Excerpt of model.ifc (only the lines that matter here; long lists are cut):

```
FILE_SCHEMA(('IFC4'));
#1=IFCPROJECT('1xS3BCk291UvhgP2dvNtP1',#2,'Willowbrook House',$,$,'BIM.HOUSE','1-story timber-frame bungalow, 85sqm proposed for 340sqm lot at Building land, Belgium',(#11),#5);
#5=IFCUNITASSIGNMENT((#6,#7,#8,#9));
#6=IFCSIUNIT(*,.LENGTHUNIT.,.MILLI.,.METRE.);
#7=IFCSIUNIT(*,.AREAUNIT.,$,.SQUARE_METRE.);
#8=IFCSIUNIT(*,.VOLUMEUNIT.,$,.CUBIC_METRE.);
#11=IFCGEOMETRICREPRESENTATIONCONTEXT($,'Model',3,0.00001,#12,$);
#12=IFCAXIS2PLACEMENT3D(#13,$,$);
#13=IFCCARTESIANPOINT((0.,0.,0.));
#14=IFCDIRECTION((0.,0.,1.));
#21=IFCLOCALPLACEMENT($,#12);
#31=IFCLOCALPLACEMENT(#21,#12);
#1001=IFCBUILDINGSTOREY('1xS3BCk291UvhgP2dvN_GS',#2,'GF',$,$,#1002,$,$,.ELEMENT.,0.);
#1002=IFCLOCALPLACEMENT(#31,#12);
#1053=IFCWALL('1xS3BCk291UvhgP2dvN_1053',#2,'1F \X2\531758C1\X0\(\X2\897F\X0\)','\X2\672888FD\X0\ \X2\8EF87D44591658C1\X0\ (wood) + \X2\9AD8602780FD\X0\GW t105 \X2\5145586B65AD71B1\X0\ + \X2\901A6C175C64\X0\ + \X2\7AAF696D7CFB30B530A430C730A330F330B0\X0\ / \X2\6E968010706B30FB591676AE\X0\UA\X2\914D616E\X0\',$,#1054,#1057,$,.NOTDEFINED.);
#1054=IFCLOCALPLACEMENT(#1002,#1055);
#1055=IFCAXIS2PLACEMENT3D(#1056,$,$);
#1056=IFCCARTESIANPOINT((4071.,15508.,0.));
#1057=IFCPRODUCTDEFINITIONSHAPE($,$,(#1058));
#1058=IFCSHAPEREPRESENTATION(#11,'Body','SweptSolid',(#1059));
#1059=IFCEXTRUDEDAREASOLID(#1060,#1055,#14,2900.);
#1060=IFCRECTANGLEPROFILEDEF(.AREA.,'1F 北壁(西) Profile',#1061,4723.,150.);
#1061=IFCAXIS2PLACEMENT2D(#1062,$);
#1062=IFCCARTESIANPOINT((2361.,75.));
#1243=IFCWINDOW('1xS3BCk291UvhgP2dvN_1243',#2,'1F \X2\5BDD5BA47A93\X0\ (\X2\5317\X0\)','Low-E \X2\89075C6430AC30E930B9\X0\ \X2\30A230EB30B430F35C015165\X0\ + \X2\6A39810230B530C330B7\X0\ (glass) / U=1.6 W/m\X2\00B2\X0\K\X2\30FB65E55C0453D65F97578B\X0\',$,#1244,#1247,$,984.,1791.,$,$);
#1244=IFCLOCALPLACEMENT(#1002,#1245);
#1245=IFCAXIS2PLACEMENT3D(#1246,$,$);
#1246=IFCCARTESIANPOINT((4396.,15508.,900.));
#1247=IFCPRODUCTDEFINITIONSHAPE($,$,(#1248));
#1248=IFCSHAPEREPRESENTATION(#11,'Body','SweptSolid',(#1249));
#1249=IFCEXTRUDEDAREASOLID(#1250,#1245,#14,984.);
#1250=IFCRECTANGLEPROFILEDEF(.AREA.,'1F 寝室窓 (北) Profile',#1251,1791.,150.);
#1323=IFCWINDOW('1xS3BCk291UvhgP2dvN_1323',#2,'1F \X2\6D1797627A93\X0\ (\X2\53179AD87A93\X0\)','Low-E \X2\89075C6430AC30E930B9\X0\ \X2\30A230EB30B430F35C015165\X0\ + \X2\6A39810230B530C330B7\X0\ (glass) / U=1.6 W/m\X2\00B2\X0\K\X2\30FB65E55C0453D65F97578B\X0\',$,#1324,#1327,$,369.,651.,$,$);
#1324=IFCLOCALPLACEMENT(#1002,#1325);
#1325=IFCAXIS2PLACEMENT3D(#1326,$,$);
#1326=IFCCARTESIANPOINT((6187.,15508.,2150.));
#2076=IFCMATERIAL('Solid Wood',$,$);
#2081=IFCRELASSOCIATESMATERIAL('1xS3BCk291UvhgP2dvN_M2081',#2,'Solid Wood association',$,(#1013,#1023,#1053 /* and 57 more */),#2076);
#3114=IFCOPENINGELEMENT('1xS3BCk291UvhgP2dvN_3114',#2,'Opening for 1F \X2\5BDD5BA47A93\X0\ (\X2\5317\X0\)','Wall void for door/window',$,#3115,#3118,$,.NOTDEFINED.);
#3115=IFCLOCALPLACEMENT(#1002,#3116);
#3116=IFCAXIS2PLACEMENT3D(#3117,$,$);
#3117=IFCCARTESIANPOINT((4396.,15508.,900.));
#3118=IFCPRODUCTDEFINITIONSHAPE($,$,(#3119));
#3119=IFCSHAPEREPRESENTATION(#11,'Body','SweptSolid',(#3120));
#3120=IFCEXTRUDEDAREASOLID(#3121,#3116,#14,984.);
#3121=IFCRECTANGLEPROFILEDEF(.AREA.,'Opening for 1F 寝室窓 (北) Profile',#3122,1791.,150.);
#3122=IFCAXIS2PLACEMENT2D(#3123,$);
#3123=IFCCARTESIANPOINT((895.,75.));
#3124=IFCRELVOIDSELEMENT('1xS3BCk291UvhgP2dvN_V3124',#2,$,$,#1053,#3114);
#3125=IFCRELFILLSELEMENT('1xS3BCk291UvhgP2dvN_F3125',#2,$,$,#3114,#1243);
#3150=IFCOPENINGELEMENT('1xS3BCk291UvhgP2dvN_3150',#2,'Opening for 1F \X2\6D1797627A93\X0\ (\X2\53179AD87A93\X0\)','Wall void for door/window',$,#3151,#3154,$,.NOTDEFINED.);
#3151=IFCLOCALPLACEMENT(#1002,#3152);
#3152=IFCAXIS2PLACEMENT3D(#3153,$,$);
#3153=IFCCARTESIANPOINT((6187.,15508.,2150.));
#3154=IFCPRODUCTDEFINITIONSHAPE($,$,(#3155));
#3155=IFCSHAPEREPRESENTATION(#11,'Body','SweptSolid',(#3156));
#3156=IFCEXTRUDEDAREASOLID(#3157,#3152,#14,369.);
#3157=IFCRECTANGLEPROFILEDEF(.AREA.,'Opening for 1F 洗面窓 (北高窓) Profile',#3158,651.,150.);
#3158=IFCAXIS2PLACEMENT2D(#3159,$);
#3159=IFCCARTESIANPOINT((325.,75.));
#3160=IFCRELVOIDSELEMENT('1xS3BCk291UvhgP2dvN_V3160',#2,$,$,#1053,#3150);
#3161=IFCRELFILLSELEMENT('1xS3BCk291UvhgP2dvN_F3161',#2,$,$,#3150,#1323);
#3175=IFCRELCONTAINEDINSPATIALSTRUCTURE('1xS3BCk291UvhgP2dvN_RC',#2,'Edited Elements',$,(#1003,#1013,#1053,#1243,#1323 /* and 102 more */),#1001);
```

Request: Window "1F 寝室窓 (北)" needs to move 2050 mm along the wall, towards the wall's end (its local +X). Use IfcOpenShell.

```python
import ifcopenshell
import ifcopenshell.api.geometry
import ifcopenshell.util.placement
import ifcopenshell.util.unit

model = ifcopenshell.open("model.ifc")
unit_scale = ifcopenshell.util.unit.calculate_unit_scale(model)

window = model.by_guid("1xS3BCk291UvhgP2dvN_1243")
opening = window.FillsVoids[0].RelatingOpeningElement
wall = opening.VoidsElements[0].RelatingBuildingElement

wall_matrix = ifcopenshell.util.placement.get_local_placement(wall.ObjectPlacement)
shift = wall_matrix[:3, 0] * 2.05 / unit_scale
before = ifcopenshell.util.placement.get_local_placement(window.ObjectPlacement)[:3, 3].copy()

# The window is not placed relative to its opening, so move both.
for product in (opening, window):
    matrix = ifcopenshell.util.placement.get_local_placement(product.ObjectPlacement)
    matrix[:3, 3] += shift
    ifcopenshell.api.geometry.edit_object_placement(model, product=product, matrix=matrix, is_si=False)

after = ifcopenshell.util.placement.get_local_placement(window.ObjectPlacement)[:3, 3]
print("window moved by", (after - before).round(3) + 0.0)

model.write("model_edited.ifc")
```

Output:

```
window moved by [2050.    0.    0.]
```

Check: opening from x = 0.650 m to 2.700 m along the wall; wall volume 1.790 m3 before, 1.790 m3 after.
